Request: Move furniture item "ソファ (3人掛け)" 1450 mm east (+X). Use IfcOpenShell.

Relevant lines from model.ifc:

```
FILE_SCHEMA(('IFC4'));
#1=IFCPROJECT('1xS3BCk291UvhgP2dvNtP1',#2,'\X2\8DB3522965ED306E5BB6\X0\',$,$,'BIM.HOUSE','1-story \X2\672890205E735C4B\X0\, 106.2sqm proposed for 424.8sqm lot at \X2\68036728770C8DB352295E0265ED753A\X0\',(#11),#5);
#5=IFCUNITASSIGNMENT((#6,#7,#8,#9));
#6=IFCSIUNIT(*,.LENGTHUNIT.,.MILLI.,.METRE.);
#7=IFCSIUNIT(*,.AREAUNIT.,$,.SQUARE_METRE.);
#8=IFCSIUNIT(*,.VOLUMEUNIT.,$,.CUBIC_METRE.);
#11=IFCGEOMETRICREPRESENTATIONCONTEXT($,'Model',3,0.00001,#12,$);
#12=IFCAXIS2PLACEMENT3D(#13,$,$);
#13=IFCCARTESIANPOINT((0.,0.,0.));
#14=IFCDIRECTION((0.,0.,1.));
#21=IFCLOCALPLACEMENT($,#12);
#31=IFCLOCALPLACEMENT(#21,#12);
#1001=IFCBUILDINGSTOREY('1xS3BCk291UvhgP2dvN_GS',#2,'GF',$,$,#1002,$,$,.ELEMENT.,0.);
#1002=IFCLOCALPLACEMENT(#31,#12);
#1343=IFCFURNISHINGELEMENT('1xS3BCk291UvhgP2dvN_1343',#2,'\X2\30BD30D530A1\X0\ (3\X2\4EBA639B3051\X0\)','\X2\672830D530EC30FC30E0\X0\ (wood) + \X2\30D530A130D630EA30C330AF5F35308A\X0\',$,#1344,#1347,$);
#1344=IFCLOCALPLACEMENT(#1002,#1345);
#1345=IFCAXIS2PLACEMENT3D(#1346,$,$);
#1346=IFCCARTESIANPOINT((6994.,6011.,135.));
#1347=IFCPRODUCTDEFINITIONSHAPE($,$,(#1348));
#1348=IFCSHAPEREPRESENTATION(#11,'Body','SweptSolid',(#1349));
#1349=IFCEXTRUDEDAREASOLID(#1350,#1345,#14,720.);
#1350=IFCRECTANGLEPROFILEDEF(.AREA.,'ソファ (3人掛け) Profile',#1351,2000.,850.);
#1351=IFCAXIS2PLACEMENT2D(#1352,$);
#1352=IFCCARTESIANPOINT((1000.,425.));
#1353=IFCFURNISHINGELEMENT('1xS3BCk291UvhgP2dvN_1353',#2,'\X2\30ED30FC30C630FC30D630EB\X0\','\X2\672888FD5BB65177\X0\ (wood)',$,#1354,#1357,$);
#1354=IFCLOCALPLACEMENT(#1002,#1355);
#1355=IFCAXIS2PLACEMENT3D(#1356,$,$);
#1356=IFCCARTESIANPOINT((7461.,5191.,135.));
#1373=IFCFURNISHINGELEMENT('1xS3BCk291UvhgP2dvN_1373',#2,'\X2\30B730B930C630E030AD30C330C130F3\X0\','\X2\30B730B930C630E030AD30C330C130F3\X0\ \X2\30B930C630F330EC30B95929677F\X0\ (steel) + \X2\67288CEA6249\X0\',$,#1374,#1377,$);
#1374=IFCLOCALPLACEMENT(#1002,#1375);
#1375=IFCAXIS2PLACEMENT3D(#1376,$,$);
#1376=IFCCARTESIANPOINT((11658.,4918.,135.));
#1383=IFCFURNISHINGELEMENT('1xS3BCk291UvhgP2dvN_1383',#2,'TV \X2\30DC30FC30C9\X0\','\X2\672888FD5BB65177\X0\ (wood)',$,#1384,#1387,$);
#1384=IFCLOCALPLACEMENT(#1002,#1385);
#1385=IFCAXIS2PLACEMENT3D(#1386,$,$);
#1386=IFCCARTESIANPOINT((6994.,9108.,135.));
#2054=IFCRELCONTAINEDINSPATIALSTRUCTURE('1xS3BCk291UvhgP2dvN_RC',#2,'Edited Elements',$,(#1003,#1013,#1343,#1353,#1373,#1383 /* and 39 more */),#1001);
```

```python
import ifcopenshell
import ifcopenshell.api.geometry
import ifcopenshell.util.placement
import ifcopenshell.util.unit

model = ifcopenshell.open("model.ifc")
unit_scale = ifcopenshell.util.unit.calculate_unit_scale(model)

item = model.by_id(1343)
matrix = ifcopenshell.util.placement.get_local_placement(item.ObjectPlacement)
matrix[0, 3] += 1.45 / unit_scale
ifcopenshell.api.geometry.edit_object_placement(model, product=item, matrix=matrix, is_si=False)

print(ifcopenshell.util.placement.get_local_placement(item.ObjectPlacement).round(3) + 0.0)

model.write("model_v2.ifc")
```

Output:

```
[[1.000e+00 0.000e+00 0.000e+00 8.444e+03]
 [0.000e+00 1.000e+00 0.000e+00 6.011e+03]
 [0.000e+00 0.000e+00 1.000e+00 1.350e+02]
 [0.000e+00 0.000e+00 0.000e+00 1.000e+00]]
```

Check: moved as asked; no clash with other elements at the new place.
